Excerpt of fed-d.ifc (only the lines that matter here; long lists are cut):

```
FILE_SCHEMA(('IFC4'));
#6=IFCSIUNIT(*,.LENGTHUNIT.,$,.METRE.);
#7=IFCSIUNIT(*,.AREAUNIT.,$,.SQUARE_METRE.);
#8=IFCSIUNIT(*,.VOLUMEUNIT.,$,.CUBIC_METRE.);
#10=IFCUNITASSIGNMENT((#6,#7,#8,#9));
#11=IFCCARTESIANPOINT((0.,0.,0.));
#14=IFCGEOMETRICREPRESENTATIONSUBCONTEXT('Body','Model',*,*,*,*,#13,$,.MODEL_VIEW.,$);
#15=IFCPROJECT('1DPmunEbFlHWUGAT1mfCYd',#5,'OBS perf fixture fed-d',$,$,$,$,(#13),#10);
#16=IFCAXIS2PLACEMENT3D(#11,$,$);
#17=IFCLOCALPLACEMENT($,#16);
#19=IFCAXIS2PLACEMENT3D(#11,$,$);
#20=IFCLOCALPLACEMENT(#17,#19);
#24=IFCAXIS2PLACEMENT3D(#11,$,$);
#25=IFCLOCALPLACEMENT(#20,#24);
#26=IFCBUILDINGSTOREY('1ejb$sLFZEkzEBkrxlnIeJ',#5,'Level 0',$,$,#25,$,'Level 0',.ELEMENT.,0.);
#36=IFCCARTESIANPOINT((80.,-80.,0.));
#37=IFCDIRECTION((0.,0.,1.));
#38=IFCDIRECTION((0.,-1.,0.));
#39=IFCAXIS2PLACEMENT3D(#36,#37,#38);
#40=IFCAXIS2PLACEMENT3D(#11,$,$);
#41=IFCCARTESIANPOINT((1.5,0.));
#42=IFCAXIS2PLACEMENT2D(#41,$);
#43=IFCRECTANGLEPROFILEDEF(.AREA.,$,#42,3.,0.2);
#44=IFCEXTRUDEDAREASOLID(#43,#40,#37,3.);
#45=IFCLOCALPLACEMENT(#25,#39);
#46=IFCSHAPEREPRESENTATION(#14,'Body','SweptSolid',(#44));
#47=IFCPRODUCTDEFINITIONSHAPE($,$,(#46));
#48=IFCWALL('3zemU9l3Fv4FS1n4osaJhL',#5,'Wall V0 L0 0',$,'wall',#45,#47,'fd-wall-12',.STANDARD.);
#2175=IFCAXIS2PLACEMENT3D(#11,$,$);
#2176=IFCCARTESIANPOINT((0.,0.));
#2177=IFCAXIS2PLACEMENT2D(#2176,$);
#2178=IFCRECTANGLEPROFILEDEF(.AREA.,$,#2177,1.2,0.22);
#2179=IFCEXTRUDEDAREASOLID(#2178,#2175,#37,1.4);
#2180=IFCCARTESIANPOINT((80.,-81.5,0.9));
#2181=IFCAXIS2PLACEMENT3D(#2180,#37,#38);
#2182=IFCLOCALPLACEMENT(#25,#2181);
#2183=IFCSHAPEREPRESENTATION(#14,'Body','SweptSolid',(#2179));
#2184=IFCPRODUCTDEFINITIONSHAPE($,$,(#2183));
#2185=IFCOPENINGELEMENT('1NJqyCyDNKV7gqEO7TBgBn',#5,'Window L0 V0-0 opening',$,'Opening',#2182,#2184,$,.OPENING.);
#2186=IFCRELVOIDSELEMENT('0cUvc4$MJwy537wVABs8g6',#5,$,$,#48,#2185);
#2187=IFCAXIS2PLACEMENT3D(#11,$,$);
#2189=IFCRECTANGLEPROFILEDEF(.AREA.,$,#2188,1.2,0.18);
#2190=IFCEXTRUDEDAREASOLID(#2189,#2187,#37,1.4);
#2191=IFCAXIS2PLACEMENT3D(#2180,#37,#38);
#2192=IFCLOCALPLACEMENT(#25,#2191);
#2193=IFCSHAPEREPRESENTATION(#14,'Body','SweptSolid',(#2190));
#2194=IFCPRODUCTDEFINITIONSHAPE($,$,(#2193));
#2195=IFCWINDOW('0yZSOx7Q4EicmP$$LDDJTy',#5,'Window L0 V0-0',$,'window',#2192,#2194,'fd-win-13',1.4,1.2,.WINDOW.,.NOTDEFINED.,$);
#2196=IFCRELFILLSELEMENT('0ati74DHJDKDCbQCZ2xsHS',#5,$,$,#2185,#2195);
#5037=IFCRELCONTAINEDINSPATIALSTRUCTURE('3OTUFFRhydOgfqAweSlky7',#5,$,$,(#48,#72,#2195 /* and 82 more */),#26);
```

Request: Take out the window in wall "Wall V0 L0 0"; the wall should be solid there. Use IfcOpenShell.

```python
import ifcopenshell
import ifcopenshell.api.feature
import ifcopenshell.api.root
import ifcopenshell.geom
import ifcopenshell.util.shape

model = ifcopenshell.open("fed-d.ifc")
settings = ifcopenshell.geom.settings()


def volume(element):
    """Net volume in cubic metres, openings subtracted."""
    shape = ifcopenshell.geom.create_shape(settings, element)
    return ifcopenshell.util.shape.get_volume(shape.geometry)


window = model.by_id(2195)
opening = window.FillsVoids[0].RelatingOpeningElement
wall = opening.VoidsElements[0].RelatingBuildingElement
before = volume(wall)

ifcopenshell.api.root.remove_product(model, product=window)
ifcopenshell.api.feature.remove_feature(model, feature=opening)

after = volume(wall)

print(f"wall volume {before:.3f} -> {after:.3f} m3")

model.write("fed-d_updated.ifc")
```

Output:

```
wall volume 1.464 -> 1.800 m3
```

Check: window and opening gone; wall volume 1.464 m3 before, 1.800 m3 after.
